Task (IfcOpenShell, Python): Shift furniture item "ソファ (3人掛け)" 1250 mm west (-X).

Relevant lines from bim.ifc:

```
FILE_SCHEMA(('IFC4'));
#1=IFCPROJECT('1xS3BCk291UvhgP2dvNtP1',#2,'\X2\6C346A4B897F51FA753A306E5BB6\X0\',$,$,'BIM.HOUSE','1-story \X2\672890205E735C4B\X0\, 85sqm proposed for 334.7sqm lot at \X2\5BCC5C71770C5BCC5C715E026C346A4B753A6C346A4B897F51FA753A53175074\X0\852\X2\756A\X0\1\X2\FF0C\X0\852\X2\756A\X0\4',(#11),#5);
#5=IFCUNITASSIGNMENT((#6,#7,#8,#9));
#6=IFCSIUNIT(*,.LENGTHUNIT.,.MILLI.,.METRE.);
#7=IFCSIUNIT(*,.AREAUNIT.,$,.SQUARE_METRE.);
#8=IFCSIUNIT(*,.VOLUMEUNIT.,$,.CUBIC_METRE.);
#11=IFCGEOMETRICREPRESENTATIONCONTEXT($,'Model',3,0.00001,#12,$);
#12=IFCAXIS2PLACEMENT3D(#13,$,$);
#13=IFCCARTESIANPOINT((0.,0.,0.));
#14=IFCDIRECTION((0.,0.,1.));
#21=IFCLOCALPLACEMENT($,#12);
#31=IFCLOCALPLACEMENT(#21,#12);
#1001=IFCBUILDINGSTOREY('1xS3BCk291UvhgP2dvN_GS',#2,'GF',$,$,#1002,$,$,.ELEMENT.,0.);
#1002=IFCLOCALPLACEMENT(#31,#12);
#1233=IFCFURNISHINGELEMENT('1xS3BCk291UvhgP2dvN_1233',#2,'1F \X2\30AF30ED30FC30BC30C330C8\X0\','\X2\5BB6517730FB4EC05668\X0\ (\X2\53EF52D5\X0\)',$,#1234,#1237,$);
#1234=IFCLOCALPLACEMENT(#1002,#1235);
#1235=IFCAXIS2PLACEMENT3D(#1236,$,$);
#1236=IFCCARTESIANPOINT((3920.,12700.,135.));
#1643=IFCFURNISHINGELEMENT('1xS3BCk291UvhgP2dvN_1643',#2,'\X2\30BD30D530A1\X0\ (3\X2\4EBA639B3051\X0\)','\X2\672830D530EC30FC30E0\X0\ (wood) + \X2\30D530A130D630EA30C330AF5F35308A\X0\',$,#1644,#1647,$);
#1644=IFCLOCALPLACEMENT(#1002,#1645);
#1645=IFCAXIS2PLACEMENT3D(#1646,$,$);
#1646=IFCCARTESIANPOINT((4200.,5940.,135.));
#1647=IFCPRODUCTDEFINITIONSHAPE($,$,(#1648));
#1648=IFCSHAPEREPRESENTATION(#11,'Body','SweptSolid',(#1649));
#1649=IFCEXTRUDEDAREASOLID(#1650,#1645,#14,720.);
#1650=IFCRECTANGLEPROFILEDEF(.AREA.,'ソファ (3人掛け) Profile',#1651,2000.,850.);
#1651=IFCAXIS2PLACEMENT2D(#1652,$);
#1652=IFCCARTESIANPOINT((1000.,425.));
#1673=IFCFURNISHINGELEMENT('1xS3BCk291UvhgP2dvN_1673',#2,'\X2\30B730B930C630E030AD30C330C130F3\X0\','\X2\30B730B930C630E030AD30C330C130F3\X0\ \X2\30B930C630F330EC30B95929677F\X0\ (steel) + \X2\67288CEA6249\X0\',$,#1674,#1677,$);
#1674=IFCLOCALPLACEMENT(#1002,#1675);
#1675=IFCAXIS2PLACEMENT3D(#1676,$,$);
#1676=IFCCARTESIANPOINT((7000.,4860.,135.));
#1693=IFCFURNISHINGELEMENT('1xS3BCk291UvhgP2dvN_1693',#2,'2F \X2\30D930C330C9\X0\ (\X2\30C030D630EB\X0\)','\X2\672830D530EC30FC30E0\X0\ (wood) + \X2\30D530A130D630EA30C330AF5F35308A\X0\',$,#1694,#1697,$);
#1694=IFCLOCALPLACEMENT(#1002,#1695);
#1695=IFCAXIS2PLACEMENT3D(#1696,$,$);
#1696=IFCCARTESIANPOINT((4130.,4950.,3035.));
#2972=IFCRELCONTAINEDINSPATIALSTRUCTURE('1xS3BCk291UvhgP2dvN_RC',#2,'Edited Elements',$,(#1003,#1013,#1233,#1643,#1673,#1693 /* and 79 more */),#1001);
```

```python
import ifcopenshell
import ifcopenshell.api.geometry
import ifcopenshell.util.placement

model = ifcopenshell.open("bim.ifc")

item = model.by_guid("1xS3BCk291UvhgP2dvN_1643")
matrix = ifcopenshell.util.placement.get_local_placement(item.ObjectPlacement)
matrix[0, 3] -= 1250.0
ifcopenshell.api.geometry.edit_object_placement(model, product=item, matrix=matrix, is_si=False)

print(ifcopenshell.util.placement.get_local_placement(item.ObjectPlacement).round(3) + 0.0)

model.write("bim_edited.ifc")
```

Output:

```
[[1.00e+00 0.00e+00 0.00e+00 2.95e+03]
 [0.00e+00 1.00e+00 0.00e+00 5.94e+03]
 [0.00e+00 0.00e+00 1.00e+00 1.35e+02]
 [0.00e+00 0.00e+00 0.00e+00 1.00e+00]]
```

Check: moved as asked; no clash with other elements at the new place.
